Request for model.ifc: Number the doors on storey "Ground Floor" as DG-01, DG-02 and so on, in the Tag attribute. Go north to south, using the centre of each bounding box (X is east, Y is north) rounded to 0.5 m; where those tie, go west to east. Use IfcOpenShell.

First a look at what the model holds.

```python
import ifcopenshell
import ifcopenshell.util.element
import ifcopenshell.util.placement

model = ifcopenshell.open("model.ifc")
print(model.schema)
storey = next(s for s in model.by_type("IfcBuildingStorey") if s.Name == "Ground Floor")
doors = [e for e in ifcopenshell.util.element.get_decomposition(storey) if e.is_a("IfcDoor")]
for e in sorted(doors, key=lambda e: e.id()):
    origin = ifcopenshell.util.placement.get_local_placement(e.ObjectPlacement)[:3, 3]
    print(e.id(), e.Tag, e.Name, origin.round(2) + 0.0, sep=" | ")
```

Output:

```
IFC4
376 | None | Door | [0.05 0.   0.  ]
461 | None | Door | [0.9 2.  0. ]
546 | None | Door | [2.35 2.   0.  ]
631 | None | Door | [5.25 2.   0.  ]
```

```python
import ifcopenshell
import ifcopenshell.geom
import ifcopenshell.util.element
import ifcopenshell.util.shape

model = ifcopenshell.open("model.ifc")
settings = ifcopenshell.geom.settings()
settings.set("use-world-coords", True)


def centre(element):
    shape = ifcopenshell.geom.create_shape(settings, element)
    return ifcopenshell.util.shape.get_bbox_centroid(shape.geometry)


storey = next(s for s in model.by_type("IfcBuildingStorey") if s.Name == "Ground Floor")
doors = [e for e in ifcopenshell.util.element.get_decomposition(storey) if e.is_a("IfcDoor")]

# Insertion points can sit at a corner or the storey origin, so sort by the geometry (in metres).
centres = {e: centre(e) for e in doors}
doors.sort(key=lambda e: (-round(centres[e][1] / 0.5), centres[e][0]))

for i, e in enumerate(doors, start=1):
    number = f"DG-{i:02d}"
    e.Tag = number
    print(e.id(), number)

model.write("model_v2.ifc")
```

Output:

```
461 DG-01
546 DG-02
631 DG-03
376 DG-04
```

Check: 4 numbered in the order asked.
